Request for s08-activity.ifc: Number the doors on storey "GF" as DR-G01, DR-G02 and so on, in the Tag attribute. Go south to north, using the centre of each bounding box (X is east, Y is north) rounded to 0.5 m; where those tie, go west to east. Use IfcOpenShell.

First a look at what the model holds.

```python
import ifcopenshell
import ifcopenshell.util.element
import ifcopenshell.util.placement

model = ifcopenshell.open("s08-activity.ifc")
print(model.schema)
storey = next(s for s in model.by_type("IfcBuildingStorey") if s.Name == "GF")
doors = [e for e in ifcopenshell.util.element.get_decomposition(storey) if e.is_a("IfcDoor")]
for e in sorted(doors, key=lambda e: e.id()):
    origin = ifcopenshell.util.placement.get_local_placement(e.ObjectPlacement)[:3, 3]
    print(e.id(), e.Tag, e.Name, origin.round(2) + 0.0, sep=" | ")
```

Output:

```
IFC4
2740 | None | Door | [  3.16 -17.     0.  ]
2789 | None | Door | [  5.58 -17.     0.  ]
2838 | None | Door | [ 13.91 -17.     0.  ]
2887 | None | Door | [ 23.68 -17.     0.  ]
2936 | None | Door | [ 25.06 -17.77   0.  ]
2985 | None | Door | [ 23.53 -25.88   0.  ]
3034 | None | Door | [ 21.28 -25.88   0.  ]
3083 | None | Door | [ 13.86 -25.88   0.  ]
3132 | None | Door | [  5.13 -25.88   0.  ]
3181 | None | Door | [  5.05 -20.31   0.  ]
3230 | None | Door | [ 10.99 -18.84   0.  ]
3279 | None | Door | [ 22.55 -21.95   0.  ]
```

```python
import ifcopenshell
import ifcopenshell.geom
import ifcopenshell.util.element
import ifcopenshell.util.shape

model = ifcopenshell.open("s08-activity.ifc")
settings = ifcopenshell.geom.settings()
settings.set("use-world-coords", True)


def centre(element):
    shape = ifcopenshell.geom.create_shape(settings, element)
    return ifcopenshell.util.shape.get_bbox_centroid(shape.geometry)


storey = next(s for s in model.by_type("IfcBuildingStorey") if s.Name == "GF")
doors = [e for e in ifcopenshell.util.element.get_decomposition(storey) if e.is_a("IfcDoor")]

# Insertion points can sit at a corner or the storey origin, so sort by the geometry (in metres).
centres = {e: centre(e) for e in doors}
doors.sort(key=lambda e: (round(centres[e][1] / 0.5), centres[e][0]))

for i, e in enumerate(doors, start=1):
    number = f"DR-G{i:02d}"
    e.Tag = number
    print(e.id(), number)

model.write("s08-activity_edited.ifc")
```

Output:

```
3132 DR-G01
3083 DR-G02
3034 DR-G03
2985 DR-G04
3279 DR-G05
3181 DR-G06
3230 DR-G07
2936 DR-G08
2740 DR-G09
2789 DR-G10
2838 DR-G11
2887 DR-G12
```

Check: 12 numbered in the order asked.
